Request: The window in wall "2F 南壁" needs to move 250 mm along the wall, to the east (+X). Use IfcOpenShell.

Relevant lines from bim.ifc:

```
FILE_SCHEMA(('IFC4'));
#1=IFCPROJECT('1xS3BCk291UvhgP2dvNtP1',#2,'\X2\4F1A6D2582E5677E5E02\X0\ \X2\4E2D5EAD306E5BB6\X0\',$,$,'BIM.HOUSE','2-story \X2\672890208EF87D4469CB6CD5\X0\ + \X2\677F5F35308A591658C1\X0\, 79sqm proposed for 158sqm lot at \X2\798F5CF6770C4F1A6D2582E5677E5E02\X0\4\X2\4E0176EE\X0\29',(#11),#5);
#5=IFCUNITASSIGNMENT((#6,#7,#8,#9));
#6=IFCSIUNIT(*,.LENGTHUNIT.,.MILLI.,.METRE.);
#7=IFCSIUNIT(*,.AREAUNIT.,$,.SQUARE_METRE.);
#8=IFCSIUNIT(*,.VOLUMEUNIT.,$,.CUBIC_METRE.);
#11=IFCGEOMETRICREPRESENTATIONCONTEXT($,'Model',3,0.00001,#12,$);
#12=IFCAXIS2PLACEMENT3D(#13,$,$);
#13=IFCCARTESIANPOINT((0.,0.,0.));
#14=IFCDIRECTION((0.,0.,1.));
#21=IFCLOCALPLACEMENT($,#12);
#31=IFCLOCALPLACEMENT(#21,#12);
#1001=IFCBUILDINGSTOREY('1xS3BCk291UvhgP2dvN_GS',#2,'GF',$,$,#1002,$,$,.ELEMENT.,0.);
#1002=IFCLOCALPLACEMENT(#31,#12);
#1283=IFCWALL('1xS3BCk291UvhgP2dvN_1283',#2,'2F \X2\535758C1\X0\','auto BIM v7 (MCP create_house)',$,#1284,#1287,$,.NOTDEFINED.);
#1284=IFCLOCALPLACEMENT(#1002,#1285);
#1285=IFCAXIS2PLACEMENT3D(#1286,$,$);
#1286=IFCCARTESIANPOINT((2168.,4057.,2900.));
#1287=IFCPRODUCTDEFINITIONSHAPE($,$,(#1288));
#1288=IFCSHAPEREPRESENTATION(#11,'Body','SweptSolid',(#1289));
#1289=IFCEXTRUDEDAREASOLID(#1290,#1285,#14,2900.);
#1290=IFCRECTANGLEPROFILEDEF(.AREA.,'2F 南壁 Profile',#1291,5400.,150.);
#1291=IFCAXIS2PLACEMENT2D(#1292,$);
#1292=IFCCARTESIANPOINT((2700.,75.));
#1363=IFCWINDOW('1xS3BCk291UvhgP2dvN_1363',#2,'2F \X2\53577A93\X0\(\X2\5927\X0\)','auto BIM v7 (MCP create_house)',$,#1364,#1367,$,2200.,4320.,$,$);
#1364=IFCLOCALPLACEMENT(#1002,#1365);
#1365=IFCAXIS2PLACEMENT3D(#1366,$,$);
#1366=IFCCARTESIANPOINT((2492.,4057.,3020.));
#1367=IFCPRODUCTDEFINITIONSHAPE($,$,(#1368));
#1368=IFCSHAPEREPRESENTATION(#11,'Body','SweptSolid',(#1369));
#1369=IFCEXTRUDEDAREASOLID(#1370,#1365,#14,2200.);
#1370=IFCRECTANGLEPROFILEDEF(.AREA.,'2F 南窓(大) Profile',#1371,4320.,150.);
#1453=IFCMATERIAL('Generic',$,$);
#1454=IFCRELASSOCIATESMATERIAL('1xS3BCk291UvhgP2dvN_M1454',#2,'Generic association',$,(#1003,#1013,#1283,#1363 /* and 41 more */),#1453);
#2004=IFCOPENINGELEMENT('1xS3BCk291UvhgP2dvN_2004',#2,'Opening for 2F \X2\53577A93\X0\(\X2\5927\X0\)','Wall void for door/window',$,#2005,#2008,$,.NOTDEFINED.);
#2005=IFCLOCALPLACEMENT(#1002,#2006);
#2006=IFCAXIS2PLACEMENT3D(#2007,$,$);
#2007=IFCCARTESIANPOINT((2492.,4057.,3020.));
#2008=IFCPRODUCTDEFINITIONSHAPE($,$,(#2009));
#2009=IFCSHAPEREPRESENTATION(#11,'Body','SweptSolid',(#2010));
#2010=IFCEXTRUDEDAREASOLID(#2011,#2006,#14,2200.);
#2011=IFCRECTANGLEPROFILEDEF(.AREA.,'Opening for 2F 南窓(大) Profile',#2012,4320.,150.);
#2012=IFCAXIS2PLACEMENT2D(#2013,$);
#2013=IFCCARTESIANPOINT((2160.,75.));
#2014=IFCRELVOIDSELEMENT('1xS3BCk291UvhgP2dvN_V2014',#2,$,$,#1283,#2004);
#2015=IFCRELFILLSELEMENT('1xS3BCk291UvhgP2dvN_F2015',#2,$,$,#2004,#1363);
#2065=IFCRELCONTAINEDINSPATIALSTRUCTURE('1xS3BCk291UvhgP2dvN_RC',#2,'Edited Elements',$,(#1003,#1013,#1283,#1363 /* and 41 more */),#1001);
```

```python
import ifcopenshell
import ifcopenshell.api.geometry
import ifcopenshell.util.placement
import ifcopenshell.util.unit

model = ifcopenshell.open("bim.ifc")
unit_scale = ifcopenshell.util.unit.calculate_unit_scale(model)

window = model.by_id(1363)
opening = window.FillsVoids[0].RelatingOpeningElement
wall = opening.VoidsElements[0].RelatingBuildingElement

wall_matrix = ifcopenshell.util.placement.get_local_placement(wall.ObjectPlacement)
shift = wall_matrix[:3, 0] * 0.25 / unit_scale
before = ifcopenshell.util.placement.get_local_placement(window.ObjectPlacement)[:3, 3].copy()

# The window is not placed relative to its opening, so move both.
for product in (opening, window):
    matrix = ifcopenshell.util.placement.get_local_placement(product.ObjectPlacement)
    matrix[:3, 3] += shift
    ifcopenshell.api.geometry.edit_object_placement(model, product=product, matrix=matrix, is_si=False)

after = ifcopenshell.util.placement.get_local_placement(window.ObjectPlacement)[:3, 3]
print("window moved by", (after - before).round(3) + 0.0)

model.write("bim_v2.ifc")
```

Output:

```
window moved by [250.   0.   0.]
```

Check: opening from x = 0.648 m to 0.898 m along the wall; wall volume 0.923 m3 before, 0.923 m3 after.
